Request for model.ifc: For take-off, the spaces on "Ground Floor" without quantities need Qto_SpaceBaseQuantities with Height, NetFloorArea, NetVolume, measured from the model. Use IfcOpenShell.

First a look at what the model holds.

```python
import ifcopenshell
import ifcopenshell.util.element
import ifcopenshell.util.unit

model = ifcopenshell.open("model.ifc")
print(model.schema)
for unit_type in ("LENGTHUNIT", "AREAUNIT", "VOLUMEUNIT"):
    print(unit_type, ifcopenshell.util.unit.calculate_unit_scale(model, unit_type))
storey = next(s for s in model.by_type("IfcBuildingStorey") if s.Name == "Ground Floor")
spaces = [e for e in ifcopenshell.util.element.get_decomposition(storey) if e.is_a("IfcSpace")]
for e in sorted(spaces, key=lambda e: e.id()):
    print(e.id(), e.is_a(), e.Name, list(ifcopenshell.util.element.get_psets(e, qtos_only=True)), sep=" | ")
```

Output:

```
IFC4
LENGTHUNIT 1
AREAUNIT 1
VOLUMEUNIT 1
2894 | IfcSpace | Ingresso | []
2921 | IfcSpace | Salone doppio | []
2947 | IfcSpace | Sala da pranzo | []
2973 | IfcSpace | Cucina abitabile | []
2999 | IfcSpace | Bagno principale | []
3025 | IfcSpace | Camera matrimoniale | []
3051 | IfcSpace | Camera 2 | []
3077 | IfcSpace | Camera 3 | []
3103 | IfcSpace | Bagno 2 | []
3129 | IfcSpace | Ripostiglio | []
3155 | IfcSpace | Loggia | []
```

```python
import ifcopenshell
import ifcopenshell.api.pset
import ifcopenshell.geom
import ifcopenshell.util.element
import ifcopenshell.util.shape
import ifcopenshell.util.unit

model = ifcopenshell.open("model.ifc")
unit_scale = ifcopenshell.util.unit.calculate_unit_scale(model)
area_scale = ifcopenshell.util.unit.calculate_unit_scale(model, "AREAUNIT")
volume_scale = ifcopenshell.util.unit.calculate_unit_scale(model, "VOLUMEUNIT")
settings = ifcopenshell.geom.settings()

storey = next(s for s in model.by_type("IfcBuildingStorey") if s.Name == "Ground Floor")
spaces = [e for e in ifcopenshell.util.element.get_decomposition(storey) if e.is_a("IfcSpace")]

for e in sorted(spaces, key=lambda e: e.id()):
    if ifcopenshell.util.element.get_psets(e, qtos_only=True, should_inherit=False):
        continue
    # Geometry comes back in metres, in the element's own axes.
    shape = ifcopenshell.geom.create_shape(settings, e)
    values = {
        "Height": ifcopenshell.util.shape.get_z(shape.geometry) / unit_scale,
        "NetFloorArea": ifcopenshell.util.shape.get_footprint_area(shape.geometry) / area_scale,
        "NetVolume": ifcopenshell.util.shape.get_volume(shape.geometry) / volume_scale,
    }
    qto = ifcopenshell.api.pset.add_qto(model, product=e, name="Qto_SpaceBaseQuantities")
    ifcopenshell.api.pset.edit_qto(model, qto=qto, properties=values)
    print(e.id(), {k: round(v, 3) for k, v in values.items()})

model.write("model_v2.ifc")
```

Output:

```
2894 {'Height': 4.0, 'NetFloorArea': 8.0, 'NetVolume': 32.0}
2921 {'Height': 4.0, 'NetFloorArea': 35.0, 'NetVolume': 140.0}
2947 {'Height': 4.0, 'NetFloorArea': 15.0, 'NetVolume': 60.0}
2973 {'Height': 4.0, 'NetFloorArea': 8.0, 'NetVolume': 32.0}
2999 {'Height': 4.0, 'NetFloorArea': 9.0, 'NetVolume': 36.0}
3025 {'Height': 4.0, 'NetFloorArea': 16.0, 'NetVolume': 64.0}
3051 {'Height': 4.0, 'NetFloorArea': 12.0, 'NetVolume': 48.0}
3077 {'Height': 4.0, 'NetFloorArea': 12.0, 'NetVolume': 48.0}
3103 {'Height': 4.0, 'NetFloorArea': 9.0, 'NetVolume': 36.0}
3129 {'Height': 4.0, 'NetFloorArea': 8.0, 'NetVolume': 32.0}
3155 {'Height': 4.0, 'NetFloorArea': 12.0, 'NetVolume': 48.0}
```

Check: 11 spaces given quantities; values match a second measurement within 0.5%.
